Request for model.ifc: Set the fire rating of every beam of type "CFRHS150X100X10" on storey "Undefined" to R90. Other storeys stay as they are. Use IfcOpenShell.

First a look at what the model holds.

```python
import ifcopenshell
import ifcopenshell.util.element

model = ifcopenshell.open("model.ifc")
print(model.schema)
storey = next(s for s in model.by_type("IfcBuildingStorey") if s.Name == "Undefined")
beams = [e for e in ifcopenshell.util.element.get_decomposition(storey) if e.is_a("IfcBeam")]
seen = {}
for e in beams:
    element_type = ifcopenshell.util.element.get_type(e)
    key = (element_type.Name if element_type != e and element_type else None, ifcopenshell.util.element.get_pset(e, "Pset_BeamCommon", "FireRating"))
    seen[key] = seen.get(key, 0) + 1
for (name, value), count in sorted(seen.items(), key=str):
    print(count, "x", name, "|", value)
```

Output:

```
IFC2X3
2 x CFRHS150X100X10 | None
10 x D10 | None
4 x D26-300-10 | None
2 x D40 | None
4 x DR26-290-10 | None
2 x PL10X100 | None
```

```python
import ifcopenshell
import ifcopenshell.api.pset
import ifcopenshell.util.element

model = ifcopenshell.open("model.ifc")

storey = next(s for s in model.by_type("IfcBuildingStorey") if s.Name == "Undefined")
beams = [e for e in ifcopenshell.util.element.get_decomposition(storey) if e.is_a("IfcBeam")]

count = 0
for e in beams:
    element_type = ifcopenshell.util.element.get_type(e)
    if element_type in (None, e) or element_type.Name != "CFRHS150X100X10":
        continue
    found = ifcopenshell.util.element.get_pset(e, "Pset_BeamCommon", should_inherit=False)
    if found:
        pset = model.by_id(found["id"])
        if len(ifcopenshell.util.element.get_elements_by_pset(pset)) > 1:
            pset = ifcopenshell.api.pset.unshare_pset(model, products=[e], pset=pset)[0]
    else:
        pset = ifcopenshell.api.pset.add_pset(model, product=e, name="Pset_BeamCommon")
    ifcopenshell.api.pset.edit_pset(model, pset=pset, properties={"FireRating": "R90"})
    count += 1

print(count, "beams updated")

model.write("model_rev.ifc")
```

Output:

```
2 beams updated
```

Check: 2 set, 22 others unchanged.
